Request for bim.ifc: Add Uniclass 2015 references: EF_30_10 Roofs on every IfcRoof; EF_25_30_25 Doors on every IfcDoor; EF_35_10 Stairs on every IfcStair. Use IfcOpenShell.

First a look at what the model holds.

```python
import ifcopenshell

model = ifcopenshell.open("bim.ifc")
print(model.schema)
print("classifications:", [c.Name for c in model.by_type("IfcClassification")])
for ifc_class in ("IfcDoor", "IfcRoof", "IfcStair", "IfcWall", "IfcWindow"):
    print(ifc_class, len(model.by_type(ifc_class)))
```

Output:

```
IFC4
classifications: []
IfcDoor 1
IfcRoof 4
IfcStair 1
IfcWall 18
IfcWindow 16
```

```python
import ifcopenshell
import ifcopenshell.api.classification

model = ifcopenshell.open("bim.ifc")

system = ifcopenshell.api.classification.add_classification(model, classification="Uniclass 2015")

codes = {
    "IfcRoof": ("EF_30_10", "Roofs"),
    "IfcDoor": ("EF_25_30_25", "Doors"),
    "IfcStair": ("EF_35_10", "Stairs"),
}
for ifc_class, (code, name) in codes.items():
    products = model.by_type(ifc_class)
    ifcopenshell.api.classification.add_reference(
        model, products=products, classification=system, identification=code, name=name
    )
    print(code, len(products))

model.write("bim_v2.ifc")
```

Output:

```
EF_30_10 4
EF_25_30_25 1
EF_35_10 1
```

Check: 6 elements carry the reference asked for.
